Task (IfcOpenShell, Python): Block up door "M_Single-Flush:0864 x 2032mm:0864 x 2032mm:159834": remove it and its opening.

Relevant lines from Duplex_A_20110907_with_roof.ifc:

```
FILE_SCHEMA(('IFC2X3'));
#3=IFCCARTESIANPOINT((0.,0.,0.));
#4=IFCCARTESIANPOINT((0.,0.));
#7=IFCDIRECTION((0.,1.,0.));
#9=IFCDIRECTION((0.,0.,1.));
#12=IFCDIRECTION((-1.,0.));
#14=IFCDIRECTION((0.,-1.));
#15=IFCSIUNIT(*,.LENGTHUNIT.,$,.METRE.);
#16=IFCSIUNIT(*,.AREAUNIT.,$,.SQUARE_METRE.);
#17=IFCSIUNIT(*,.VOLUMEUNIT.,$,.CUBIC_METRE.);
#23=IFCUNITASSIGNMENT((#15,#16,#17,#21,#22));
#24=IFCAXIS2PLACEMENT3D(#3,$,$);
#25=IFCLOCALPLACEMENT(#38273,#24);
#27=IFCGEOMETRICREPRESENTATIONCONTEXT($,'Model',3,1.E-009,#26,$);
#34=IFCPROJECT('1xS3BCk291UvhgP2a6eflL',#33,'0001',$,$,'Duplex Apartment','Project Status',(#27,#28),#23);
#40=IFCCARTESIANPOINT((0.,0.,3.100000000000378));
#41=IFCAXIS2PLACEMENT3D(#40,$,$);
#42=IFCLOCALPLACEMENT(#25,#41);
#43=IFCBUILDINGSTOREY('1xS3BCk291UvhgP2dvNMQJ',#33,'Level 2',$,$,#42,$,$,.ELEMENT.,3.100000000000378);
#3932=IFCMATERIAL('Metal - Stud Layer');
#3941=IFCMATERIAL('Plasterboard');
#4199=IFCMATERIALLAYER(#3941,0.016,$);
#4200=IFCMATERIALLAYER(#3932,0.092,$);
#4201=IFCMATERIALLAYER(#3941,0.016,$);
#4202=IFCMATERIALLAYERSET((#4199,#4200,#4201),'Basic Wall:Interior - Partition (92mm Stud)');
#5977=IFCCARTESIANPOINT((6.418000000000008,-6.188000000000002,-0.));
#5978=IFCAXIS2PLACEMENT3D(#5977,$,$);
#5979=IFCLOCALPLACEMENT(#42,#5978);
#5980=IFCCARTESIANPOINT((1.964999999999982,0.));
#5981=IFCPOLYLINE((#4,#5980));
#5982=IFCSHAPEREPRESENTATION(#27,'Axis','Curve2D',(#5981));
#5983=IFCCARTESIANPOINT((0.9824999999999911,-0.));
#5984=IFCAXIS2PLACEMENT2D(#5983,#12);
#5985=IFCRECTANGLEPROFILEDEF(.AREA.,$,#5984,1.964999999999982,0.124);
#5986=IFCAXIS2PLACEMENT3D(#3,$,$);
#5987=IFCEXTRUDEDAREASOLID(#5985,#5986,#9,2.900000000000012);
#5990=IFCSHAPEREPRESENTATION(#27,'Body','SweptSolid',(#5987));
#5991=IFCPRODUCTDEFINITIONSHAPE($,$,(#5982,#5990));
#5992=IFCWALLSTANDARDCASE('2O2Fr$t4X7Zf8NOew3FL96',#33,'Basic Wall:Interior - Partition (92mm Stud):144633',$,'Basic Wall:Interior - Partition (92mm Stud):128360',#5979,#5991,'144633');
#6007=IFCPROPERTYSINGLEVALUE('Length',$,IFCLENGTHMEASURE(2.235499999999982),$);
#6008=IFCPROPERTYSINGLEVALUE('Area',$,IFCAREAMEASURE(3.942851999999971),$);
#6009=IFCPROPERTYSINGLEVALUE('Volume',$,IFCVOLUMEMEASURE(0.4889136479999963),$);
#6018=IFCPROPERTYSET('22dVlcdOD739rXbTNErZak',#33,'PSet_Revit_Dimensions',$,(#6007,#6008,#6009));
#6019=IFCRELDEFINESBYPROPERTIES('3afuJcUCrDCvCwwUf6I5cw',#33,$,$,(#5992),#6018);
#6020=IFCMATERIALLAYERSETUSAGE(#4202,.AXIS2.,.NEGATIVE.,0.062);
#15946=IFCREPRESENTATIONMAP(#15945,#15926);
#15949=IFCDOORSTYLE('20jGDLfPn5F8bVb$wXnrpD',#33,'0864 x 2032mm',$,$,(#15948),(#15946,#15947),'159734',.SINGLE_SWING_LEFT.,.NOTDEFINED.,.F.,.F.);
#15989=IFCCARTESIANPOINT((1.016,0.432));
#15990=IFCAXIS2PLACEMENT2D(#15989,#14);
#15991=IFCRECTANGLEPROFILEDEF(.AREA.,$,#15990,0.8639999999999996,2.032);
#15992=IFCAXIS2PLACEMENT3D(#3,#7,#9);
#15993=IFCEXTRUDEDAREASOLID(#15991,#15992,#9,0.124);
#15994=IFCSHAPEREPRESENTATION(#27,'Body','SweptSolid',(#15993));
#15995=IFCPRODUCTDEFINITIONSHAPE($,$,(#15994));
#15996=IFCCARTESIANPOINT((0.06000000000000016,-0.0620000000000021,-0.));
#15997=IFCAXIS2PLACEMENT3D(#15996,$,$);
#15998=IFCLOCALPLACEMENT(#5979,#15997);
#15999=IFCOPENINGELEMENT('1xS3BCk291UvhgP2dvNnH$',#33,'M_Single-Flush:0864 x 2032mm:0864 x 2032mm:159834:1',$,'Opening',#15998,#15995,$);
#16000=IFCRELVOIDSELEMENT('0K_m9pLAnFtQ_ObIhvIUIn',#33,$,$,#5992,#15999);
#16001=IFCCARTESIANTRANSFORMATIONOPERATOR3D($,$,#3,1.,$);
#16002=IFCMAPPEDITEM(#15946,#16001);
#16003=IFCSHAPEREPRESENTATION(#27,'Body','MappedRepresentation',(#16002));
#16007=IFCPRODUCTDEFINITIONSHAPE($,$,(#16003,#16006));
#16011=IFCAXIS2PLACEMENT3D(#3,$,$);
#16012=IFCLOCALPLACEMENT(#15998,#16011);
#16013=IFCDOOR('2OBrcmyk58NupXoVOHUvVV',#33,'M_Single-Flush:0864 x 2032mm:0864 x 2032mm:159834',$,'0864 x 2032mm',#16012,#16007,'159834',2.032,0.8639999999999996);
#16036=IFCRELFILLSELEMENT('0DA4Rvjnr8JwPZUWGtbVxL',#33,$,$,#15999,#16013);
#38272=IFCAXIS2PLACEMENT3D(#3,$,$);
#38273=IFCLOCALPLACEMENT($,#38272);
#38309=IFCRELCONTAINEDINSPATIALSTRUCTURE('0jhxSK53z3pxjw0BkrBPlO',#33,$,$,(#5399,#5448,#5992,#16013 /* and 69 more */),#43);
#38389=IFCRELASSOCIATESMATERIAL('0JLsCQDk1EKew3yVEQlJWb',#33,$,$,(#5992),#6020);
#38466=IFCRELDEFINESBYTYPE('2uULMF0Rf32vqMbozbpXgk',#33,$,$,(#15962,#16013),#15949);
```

```python
import ifcopenshell
import ifcopenshell.api.feature
import ifcopenshell.api.pset
import ifcopenshell.api.root
import ifcopenshell.geom
import ifcopenshell.util.element
import ifcopenshell.util.shape
import ifcopenshell.util.unit

model = ifcopenshell.open("Duplex_A_20110907_with_roof.ifc")
area_scale = ifcopenshell.util.unit.calculate_unit_scale(model, "AREAUNIT")
volume_scale = ifcopenshell.util.unit.calculate_unit_scale(model, "VOLUMEUNIT")
settings = ifcopenshell.geom.settings()


def volume(element):
    """Net volume in cubic metres, openings subtracted."""
    shape = ifcopenshell.geom.create_shape(settings, element)
    return ifcopenshell.util.shape.get_volume(shape.geometry)


door = model.by_guid("2OBrcmyk58NupXoVOHUvVV")
opening = door.FillsVoids[0].RelatingOpeningElement
wall = opening.VoidsElements[0].RelatingBuildingElement
before = volume(wall)

ifcopenshell.api.root.remove_product(model, product=door)
ifcopenshell.api.feature.remove_feature(model, feature=opening)

after = volume(wall)
thickness = 0.124  # wall thickness in metres

# Update the wall's stored quantities.
pset = model.by_id(ifcopenshell.util.element.get_pset(wall, "PSet_Revit_Dimensions", should_inherit=False)["id"])
ifcopenshell.api.pset.edit_pset(model, pset=pset, properties={
    "Area": model.create_entity("IfcAreaMeasure", after / thickness / area_scale),
    "Volume": model.create_entity("IfcVolumeMeasure", after / volume_scale),
})

print(f"wall volume {before:.3f} -> {after:.3f} m3")

model.write("Duplex_A_20110907_with_roof_v2.ifc")
```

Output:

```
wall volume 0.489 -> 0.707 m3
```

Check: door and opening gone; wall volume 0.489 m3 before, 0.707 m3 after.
